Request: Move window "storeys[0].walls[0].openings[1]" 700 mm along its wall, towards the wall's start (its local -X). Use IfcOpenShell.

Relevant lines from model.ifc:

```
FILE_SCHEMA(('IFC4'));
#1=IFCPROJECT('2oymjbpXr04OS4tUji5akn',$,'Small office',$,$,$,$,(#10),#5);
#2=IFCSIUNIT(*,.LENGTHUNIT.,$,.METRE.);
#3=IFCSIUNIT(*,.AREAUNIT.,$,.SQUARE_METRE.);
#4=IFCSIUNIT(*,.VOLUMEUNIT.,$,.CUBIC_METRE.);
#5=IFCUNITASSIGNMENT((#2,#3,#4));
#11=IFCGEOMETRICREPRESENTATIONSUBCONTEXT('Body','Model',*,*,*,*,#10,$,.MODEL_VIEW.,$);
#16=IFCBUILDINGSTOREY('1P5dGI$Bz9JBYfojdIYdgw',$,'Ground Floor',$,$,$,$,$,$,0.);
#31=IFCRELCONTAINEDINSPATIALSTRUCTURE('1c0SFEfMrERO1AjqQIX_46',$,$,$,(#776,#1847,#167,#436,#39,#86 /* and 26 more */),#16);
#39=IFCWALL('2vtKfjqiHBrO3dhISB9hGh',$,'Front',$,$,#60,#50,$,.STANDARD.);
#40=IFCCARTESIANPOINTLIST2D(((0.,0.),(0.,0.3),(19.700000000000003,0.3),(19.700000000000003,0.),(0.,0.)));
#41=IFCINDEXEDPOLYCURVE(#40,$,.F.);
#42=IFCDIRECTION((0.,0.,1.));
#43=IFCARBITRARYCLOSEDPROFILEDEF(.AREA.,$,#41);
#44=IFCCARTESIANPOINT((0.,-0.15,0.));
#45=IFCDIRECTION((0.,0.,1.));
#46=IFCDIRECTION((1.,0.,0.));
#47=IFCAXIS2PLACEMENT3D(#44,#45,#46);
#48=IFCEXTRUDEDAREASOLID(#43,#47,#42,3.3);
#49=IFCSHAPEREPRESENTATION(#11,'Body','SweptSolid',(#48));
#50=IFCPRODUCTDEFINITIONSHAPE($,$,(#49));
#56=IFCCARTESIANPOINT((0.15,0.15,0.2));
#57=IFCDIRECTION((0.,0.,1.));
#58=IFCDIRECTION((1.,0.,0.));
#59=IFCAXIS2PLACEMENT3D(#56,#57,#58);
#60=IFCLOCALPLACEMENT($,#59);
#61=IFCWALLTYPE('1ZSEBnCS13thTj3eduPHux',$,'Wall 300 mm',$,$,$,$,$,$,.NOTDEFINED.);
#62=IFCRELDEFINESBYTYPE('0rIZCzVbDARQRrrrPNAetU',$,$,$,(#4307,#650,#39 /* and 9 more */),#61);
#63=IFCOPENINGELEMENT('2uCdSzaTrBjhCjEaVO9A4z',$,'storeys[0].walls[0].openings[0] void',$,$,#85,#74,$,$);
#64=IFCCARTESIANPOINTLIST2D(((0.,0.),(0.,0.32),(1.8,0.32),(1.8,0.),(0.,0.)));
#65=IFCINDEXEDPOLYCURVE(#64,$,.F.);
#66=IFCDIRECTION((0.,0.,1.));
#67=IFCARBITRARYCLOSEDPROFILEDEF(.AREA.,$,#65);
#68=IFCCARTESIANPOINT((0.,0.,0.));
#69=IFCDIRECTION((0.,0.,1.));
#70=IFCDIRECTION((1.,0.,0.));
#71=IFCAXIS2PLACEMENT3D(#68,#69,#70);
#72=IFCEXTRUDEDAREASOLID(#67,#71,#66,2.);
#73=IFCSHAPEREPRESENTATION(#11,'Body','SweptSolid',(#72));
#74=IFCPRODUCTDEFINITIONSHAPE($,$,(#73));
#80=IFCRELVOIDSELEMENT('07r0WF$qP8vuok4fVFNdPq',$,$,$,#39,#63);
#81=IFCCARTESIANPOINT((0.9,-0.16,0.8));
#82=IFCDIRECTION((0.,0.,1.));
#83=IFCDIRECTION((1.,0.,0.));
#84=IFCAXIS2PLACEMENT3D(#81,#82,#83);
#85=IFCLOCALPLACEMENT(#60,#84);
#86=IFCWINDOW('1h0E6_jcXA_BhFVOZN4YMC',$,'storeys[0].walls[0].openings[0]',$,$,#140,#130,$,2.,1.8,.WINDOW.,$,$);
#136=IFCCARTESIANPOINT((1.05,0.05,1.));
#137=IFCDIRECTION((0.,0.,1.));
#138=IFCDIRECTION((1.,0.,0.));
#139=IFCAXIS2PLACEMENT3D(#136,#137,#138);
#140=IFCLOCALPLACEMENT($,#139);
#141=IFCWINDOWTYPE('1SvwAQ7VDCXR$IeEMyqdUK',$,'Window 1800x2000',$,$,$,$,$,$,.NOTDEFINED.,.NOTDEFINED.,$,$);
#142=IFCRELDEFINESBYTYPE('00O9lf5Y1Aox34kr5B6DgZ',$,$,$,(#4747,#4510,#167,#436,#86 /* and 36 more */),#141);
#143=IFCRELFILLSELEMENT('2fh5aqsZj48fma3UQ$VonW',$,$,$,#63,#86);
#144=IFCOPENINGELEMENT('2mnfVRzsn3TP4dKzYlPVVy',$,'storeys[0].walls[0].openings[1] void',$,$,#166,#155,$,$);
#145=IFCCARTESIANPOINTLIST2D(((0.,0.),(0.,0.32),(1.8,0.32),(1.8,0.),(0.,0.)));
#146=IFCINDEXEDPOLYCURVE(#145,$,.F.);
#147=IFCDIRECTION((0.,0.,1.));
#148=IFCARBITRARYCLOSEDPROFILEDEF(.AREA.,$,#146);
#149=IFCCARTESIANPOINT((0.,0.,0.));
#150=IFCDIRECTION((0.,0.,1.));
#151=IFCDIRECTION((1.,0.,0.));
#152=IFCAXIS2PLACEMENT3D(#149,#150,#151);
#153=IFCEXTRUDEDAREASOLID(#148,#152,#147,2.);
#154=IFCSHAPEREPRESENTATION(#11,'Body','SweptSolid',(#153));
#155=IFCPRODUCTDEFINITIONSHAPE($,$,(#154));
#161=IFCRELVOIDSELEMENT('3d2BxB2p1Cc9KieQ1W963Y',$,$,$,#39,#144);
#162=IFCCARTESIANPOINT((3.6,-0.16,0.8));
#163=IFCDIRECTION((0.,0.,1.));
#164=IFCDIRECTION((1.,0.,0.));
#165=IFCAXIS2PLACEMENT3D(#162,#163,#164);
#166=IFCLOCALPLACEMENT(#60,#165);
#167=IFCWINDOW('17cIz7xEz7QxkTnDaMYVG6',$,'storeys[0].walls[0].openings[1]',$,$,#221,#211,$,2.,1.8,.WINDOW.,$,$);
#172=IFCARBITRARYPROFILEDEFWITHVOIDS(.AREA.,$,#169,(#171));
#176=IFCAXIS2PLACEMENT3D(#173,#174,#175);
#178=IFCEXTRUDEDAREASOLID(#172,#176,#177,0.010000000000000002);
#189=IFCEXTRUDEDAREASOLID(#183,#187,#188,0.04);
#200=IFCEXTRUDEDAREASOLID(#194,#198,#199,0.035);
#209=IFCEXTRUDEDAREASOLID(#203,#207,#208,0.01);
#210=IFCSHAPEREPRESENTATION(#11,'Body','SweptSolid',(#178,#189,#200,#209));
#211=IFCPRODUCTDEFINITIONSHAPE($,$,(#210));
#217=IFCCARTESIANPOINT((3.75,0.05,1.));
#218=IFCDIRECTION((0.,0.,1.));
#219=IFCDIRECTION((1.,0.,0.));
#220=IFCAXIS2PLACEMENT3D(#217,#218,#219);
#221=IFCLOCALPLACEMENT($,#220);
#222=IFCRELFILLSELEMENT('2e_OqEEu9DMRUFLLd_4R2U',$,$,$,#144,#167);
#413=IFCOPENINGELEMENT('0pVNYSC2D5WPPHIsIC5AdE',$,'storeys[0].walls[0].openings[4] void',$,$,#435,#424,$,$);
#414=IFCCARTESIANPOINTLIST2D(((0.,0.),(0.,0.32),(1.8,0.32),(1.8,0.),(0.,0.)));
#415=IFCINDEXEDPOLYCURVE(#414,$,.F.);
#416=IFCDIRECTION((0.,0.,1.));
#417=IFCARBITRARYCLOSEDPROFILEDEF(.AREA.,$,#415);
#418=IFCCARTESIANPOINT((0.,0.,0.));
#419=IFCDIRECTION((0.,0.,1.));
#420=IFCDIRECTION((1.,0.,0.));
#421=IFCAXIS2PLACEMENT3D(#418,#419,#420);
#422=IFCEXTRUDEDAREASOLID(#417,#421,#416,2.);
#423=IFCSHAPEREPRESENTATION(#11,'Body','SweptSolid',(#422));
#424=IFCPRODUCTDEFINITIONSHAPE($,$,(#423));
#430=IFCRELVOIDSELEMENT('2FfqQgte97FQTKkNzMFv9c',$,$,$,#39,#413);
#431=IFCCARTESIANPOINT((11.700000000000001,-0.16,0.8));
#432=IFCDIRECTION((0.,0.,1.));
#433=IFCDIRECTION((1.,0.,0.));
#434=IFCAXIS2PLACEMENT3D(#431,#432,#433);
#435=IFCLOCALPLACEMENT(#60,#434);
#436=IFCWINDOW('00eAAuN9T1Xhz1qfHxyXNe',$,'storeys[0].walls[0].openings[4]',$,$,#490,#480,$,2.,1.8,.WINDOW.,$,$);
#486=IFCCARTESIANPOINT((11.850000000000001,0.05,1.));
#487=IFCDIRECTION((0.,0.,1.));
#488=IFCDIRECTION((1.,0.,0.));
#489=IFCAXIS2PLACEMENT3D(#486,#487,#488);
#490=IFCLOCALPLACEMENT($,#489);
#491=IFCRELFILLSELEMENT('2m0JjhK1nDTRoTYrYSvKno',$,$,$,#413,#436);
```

```python
import ifcopenshell
import ifcopenshell.api.geometry
import ifcopenshell.util.placement
import ifcopenshell.util.unit

model = ifcopenshell.open("model.ifc")
unit_scale = ifcopenshell.util.unit.calculate_unit_scale(model)

window = model.by_guid("17cIz7xEz7QxkTnDaMYVG6")
opening = window.FillsVoids[0].RelatingOpeningElement
wall = opening.VoidsElements[0].RelatingBuildingElement

wall_matrix = ifcopenshell.util.placement.get_local_placement(wall.ObjectPlacement)
shift = wall_matrix[:3, 0] * -0.7 / unit_scale
before = ifcopenshell.util.placement.get_local_placement(window.ObjectPlacement)[:3, 3].copy()

# The window is not placed relative to its opening, so move both.
for product in (opening, window):
    matrix = ifcopenshell.util.placement.get_local_placement(product.ObjectPlacement)
    matrix[:3, 3] += shift
    ifcopenshell.api.geometry.edit_object_placement(model, product=product, matrix=matrix, is_si=False)

after = ifcopenshell.util.placement.get_local_placement(window.ObjectPlacement)[:3, 3]
print("window moved by", (after - before).round(3) + 0.0)

model.write("model-out.ifc")
```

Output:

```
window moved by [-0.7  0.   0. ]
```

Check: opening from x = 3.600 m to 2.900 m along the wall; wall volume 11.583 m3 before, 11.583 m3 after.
